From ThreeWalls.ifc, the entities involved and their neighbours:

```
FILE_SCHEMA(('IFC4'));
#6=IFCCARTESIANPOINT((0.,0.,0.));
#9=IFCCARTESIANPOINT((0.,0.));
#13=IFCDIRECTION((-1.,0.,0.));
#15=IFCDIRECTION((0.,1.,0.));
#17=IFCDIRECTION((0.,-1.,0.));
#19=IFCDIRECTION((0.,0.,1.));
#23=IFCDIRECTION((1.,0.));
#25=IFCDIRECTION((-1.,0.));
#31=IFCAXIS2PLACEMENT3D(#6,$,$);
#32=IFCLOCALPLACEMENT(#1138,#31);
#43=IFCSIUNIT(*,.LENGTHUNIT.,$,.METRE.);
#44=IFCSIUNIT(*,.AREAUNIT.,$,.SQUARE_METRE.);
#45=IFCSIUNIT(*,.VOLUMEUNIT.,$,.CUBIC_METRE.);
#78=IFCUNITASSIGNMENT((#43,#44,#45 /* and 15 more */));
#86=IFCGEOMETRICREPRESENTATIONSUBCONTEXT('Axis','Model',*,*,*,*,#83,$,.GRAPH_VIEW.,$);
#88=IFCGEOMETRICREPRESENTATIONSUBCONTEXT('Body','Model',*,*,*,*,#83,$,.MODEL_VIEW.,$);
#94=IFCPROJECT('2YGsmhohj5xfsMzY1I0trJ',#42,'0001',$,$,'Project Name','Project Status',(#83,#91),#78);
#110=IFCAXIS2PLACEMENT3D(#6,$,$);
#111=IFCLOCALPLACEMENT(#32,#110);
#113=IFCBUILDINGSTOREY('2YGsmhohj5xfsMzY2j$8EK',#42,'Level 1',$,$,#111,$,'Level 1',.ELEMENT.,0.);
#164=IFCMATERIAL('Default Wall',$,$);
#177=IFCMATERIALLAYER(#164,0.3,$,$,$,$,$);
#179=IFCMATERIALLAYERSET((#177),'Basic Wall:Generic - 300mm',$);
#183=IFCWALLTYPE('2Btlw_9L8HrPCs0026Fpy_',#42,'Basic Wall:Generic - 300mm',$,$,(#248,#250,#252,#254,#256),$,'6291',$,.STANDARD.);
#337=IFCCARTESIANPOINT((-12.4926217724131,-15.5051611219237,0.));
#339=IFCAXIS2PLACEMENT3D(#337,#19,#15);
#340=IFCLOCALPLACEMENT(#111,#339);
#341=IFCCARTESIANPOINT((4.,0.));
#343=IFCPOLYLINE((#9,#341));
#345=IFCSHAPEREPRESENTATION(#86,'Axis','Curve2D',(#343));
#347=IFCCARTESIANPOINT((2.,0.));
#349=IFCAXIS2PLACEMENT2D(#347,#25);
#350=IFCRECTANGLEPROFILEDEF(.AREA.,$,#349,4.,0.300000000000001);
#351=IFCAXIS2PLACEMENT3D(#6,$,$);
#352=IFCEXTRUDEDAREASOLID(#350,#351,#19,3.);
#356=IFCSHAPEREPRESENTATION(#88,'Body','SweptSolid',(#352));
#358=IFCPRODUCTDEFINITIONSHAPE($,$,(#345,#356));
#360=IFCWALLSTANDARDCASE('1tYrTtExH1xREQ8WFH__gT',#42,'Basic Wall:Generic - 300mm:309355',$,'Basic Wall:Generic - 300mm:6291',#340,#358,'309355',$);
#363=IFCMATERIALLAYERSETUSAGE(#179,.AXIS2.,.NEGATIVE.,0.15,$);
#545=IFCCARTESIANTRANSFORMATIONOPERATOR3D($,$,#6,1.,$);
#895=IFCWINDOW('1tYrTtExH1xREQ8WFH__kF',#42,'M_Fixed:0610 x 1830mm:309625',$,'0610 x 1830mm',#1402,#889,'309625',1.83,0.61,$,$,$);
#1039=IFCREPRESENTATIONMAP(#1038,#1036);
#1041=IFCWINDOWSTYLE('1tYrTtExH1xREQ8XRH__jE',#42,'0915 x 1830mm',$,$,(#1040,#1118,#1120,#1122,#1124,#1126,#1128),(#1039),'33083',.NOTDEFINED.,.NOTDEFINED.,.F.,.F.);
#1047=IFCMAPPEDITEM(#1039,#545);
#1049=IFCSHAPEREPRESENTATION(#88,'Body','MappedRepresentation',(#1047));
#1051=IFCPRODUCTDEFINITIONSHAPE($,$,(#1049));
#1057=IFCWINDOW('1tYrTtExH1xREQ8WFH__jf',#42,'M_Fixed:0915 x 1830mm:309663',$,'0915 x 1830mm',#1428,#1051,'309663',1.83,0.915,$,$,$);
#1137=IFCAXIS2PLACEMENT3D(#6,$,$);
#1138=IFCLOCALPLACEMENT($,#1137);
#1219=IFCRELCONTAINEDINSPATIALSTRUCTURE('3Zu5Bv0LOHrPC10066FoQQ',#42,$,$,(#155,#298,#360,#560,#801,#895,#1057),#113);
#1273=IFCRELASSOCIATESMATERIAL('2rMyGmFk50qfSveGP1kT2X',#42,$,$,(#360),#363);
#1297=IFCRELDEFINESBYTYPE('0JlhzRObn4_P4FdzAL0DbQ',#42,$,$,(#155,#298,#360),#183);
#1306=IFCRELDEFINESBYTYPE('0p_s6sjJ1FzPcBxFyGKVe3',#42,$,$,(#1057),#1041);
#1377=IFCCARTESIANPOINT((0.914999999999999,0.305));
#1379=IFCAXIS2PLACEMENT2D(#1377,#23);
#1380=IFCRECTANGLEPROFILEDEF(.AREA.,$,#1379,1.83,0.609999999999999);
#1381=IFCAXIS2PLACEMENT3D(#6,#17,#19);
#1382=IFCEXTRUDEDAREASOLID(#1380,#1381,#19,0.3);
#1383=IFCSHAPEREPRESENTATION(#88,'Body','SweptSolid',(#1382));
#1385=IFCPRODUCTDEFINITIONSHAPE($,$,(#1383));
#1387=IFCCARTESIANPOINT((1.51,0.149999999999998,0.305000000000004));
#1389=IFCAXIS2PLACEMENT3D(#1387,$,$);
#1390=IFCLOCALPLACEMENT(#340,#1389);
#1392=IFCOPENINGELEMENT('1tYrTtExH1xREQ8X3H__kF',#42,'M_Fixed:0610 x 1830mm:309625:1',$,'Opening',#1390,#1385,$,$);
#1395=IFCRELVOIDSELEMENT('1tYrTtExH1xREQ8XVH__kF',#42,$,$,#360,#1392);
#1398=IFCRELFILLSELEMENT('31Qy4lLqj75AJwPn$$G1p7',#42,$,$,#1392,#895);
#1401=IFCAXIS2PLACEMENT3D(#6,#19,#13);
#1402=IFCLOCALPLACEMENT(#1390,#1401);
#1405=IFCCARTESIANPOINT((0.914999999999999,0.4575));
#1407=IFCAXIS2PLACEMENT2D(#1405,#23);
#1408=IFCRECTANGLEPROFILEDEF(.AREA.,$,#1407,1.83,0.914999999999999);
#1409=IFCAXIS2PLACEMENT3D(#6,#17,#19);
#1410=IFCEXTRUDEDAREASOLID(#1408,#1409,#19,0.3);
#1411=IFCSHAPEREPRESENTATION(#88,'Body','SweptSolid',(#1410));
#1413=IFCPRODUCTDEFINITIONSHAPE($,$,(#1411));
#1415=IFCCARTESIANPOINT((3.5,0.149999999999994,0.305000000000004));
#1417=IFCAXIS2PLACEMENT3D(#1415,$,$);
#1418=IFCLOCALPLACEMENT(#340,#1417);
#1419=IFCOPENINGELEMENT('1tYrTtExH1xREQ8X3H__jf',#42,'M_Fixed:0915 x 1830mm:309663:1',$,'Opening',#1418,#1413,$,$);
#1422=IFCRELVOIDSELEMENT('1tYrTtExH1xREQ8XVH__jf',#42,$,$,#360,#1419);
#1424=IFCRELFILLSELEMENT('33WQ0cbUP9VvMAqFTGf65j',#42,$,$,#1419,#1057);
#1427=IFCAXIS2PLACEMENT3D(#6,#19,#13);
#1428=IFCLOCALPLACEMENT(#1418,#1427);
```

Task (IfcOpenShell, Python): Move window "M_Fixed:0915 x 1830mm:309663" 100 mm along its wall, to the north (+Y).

```python
import ifcopenshell
import ifcopenshell.api.geometry
import ifcopenshell.util.placement
import ifcopenshell.util.unit

model = ifcopenshell.open("ThreeWalls.ifc")
unit_scale = ifcopenshell.util.unit.calculate_unit_scale(model)

window = model.by_guid("1tYrTtExH1xREQ8WFH__jf")
opening = window.FillsVoids[0].RelatingOpeningElement
wall = opening.VoidsElements[0].RelatingBuildingElement

wall_matrix = ifcopenshell.util.placement.get_local_placement(wall.ObjectPlacement)
shift = wall_matrix[:3, 0] * 0.1 / unit_scale
before = ifcopenshell.util.placement.get_local_placement(window.ObjectPlacement)[:3, 3].copy()

# The window is placed relative to its opening, so it follows when the opening moves.
matrix = ifcopenshell.util.placement.get_local_placement(opening.ObjectPlacement)
matrix[:3, 3] += shift
ifcopenshell.api.geometry.edit_object_placement(
    model, product=opening, matrix=matrix, is_si=False, should_transform_children=True
)

after = ifcopenshell.util.placement.get_local_placement(window.ObjectPlacement)[:3, 3]
print("window moved by", (after - before).round(3) + 0.0)

model.write("ThreeWalls_edited.ifc")
```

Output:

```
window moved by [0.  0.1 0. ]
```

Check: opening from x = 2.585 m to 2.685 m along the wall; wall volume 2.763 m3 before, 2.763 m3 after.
